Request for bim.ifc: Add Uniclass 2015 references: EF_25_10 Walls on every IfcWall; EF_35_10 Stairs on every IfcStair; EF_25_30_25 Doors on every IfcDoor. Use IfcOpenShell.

First a look at what the model holds.

```python
import ifcopenshell

model = ifcopenshell.open("bim.ifc")
print(model.schema)
print("classifications:", [c.Name for c in model.by_type("IfcClassification")])
for ifc_class in ("IfcDoor", "IfcRoof", "IfcStair", "IfcWall", "IfcWindow"):
    print(ifc_class, len(model.by_type(ifc_class)))
```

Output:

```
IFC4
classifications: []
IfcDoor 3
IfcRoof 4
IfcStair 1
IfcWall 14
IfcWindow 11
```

```python
import ifcopenshell
import ifcopenshell.api.classification

model = ifcopenshell.open("bim.ifc")

system = ifcopenshell.api.classification.add_classification(model, classification="Uniclass 2015")

codes = {
    "IfcWall": ("EF_25_10", "Walls"),
    "IfcStair": ("EF_35_10", "Stairs"),
    "IfcDoor": ("EF_25_30_25", "Doors"),
}
for ifc_class, (code, name) in codes.items():
    products = model.by_type(ifc_class)
    ifcopenshell.api.classification.add_reference(
        model, products=products, classification=system, identification=code, name=name
    )
    print(code, len(products))

model.write("bim_v2.ifc")
```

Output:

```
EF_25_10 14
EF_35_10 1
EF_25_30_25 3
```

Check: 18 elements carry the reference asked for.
